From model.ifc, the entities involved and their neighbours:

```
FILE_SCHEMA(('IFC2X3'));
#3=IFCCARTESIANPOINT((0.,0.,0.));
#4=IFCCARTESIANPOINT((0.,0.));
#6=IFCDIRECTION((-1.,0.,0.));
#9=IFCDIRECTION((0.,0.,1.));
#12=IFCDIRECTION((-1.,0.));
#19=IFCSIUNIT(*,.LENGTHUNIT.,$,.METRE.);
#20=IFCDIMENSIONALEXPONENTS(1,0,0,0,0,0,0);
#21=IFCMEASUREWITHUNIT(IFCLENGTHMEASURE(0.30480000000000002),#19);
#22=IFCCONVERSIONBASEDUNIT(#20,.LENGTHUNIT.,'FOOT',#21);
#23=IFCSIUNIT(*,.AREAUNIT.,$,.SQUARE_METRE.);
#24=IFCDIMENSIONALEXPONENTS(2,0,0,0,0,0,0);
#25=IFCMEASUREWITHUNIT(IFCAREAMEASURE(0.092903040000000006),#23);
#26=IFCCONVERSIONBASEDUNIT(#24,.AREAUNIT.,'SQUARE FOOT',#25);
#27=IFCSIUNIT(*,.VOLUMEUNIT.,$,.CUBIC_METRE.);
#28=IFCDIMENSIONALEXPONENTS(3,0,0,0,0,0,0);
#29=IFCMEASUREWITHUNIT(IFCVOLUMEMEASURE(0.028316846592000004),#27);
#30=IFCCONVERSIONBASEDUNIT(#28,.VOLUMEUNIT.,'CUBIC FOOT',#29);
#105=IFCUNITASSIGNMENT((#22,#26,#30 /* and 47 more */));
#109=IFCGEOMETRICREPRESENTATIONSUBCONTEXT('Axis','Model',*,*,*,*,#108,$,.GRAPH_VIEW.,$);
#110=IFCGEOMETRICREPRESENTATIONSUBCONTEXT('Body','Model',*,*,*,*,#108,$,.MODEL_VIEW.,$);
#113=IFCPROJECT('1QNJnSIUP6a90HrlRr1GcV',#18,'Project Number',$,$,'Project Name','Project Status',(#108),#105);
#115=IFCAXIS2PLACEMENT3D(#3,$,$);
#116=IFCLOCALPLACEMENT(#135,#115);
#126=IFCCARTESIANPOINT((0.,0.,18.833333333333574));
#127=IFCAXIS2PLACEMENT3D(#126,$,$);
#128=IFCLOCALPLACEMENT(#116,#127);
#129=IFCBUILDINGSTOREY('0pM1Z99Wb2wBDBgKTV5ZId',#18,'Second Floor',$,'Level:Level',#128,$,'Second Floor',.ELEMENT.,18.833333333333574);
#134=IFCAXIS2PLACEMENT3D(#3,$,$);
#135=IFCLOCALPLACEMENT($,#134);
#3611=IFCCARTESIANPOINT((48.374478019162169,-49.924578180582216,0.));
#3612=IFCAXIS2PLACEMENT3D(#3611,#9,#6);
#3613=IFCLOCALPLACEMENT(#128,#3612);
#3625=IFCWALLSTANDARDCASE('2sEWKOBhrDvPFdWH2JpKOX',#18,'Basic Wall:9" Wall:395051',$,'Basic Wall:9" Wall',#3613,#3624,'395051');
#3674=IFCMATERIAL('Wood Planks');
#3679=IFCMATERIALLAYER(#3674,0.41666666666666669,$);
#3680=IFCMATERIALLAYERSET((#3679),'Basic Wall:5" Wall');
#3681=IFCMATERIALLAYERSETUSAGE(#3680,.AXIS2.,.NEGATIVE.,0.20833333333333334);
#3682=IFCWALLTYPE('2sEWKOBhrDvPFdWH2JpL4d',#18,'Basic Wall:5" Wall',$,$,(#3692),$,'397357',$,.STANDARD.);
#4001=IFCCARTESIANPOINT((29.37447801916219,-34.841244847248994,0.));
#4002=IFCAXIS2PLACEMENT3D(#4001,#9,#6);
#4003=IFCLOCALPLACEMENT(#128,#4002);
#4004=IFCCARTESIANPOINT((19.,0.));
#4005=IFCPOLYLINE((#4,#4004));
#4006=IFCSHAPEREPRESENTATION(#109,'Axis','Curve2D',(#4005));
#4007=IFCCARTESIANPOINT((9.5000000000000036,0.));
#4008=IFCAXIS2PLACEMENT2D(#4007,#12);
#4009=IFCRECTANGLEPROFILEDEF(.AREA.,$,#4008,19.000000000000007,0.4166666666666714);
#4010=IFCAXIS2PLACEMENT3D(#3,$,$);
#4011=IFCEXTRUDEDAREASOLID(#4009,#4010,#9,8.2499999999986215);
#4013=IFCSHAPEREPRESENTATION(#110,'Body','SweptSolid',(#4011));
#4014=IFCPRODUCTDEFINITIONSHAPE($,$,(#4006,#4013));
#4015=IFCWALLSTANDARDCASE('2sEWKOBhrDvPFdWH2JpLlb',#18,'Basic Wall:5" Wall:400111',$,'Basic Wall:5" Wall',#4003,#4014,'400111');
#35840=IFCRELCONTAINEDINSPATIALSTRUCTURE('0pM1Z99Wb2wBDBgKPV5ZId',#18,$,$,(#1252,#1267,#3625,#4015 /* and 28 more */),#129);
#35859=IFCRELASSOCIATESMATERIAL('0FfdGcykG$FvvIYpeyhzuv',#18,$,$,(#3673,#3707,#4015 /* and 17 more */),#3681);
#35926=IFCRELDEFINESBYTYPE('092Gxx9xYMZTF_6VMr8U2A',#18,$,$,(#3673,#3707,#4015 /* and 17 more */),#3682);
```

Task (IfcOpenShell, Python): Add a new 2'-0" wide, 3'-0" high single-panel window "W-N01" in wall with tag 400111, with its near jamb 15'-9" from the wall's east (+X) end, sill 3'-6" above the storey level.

```python
import numpy as np
import ifcopenshell
import ifcopenshell.api.feature
import ifcopenshell.api.geometry
import ifcopenshell.api.root
import ifcopenshell.api.spatial
import ifcopenshell.api.type
import ifcopenshell.geom
import ifcopenshell.util.element
import ifcopenshell.util.placement
import ifcopenshell.util.representation
import ifcopenshell.util.shape
import ifcopenshell.util.unit

model = ifcopenshell.open("model.ifc")
unit_scale = ifcopenshell.util.unit.calculate_unit_scale(model)
settings = ifcopenshell.geom.settings()


def volume(element):
    """Net volume in cubic metres, openings subtracted."""
    shape = ifcopenshell.geom.create_shape(settings, element)
    return ifcopenshell.util.shape.get_volume(shape.geometry)


wall = model.by_id(4015)
storey = ifcopenshell.util.element.get_container(wall, ifc_class="IfcBuildingStorey")
context = ifcopenshell.util.representation.get_context(model, "Model", "Body", "MODEL_VIEW")
before = volume(wall)

width, height, from_end, sill = 0.6096, 0.9144, 4.8006, 1.0668  # metres

# The wall runs along its own X axis, and the end named is its -X end.
wall_shape = ifcopenshell.geom.create_shape(settings, wall)
x, y, z = ifcopenshell.util.shape.get_vertices(wall_shape.geometry).T
start = x.min() + from_end
face, thickness = float(y.min()), float(y.max() - y.min())
wall_matrix = ifcopenshell.util.placement.get_local_placement(wall.ObjectPlacement)
level = ifcopenshell.util.placement.get_local_placement(storey.ObjectPlacement)[2, 3]


def in_wall(x, y):
    """Placement at x, y metres in the wall's axes, at sill height."""
    matrix = wall_matrix.copy()
    matrix[:, 3] = wall_matrix @ np.array([x / unit_scale, y / unit_scale, 0.0, 1.0])
    matrix[2, 3] = level + sill / unit_scale
    return matrix


# Opening: a box that overshoots both wall faces by 50 mm.
opening = ifcopenshell.api.root.create_entity(model, ifc_class="IfcOpeningElement")
box = ifcopenshell.api.geometry.add_wall_representation(
    model, context=context, length=width, height=height, thickness=thickness + 0.1
)
ifcopenshell.api.geometry.assign_representation(model, product=opening, representation=box)
ifcopenshell.api.geometry.edit_object_placement(model, product=opening, matrix=in_wall(start, face - 0.05), is_si=False)
ifcopenshell.api.feature.add_feature(model, feature=opening, element=wall)

window = ifcopenshell.api.root.create_entity(model, ifc_class="IfcWindow", name="W-N01")
window.OverallWidth, window.OverallHeight = width / unit_scale, height / unit_scale
body = ifcopenshell.api.geometry.add_window_representation(
    model,
    context=context,
    overall_width=window.OverallWidth,
    overall_height=window.OverallHeight,
    partition_type="SINGLE_PANEL",
)
ifcopenshell.api.geometry.assign_representation(model, product=window, representation=body)
ifcopenshell.api.spatial.assign_container(model, products=[window], relating_structure=storey)
fills = ifcopenshell.api.feature.add_filling(model, opening=opening, element=window)
fills.OwnerHistory = window.OwnerHistory  # required in IFC2X3

# IFC2X3 keeps the operation on the window style.
style = ifcopenshell.api.root.create_entity(model, ifc_class="IfcWindowStyle", name="W-N01")
style.OperationType, style.ConstructionType = "SINGLE_PANEL", "NOTDEFINED"
style.ParameterTakesPrecedence = style.Sizeable = False
ifcopenshell.api.type.assign_type(model, related_objects=[window], relating_type=style)

# Centre the window in the wall's thickness.
ifcopenshell.api.geometry.edit_object_placement(model, product=window, matrix=in_wall(start, face), is_si=False)
window_shape = ifcopenshell.geom.create_shape(settings, window)
depth = ifcopenshell.util.shape.get_vertices(window_shape.geometry)[:, 1]
offset = face + thickness / 2 - (depth.min() + depth.max()) / 2
ifcopenshell.api.geometry.edit_object_placement(model, product=window, matrix=in_wall(start, offset), is_si=False)

after = volume(wall)

print(f"wall volume {before:.3f} -> {after:.3f} m3")

model.write("model_updated.ifc")
```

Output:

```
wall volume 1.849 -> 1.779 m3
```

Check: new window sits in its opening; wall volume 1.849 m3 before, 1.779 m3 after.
